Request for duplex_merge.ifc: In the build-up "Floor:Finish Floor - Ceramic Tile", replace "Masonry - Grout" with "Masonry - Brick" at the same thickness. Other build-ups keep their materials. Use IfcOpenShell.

First a look at what the model holds.

```python
import ifcopenshell
import ifcopenshell.util.element

model = ifcopenshell.open("duplex_merge.ifc")
print(model.schema)
for layer_set in model.by_type("IfcMaterialLayerSet"):
    if layer_set.LayerSetName == "Floor:Finish Floor - Ceramic Tile":
        for layer in layer_set.MaterialLayers:
            print(layer.id(), layer.Material and layer.Material.Name, layer.LayerThickness, sep=" | ")
        print(len(ifcopenshell.util.element.get_elements_by_material(model, layer_set)), "elements and types use it")
print(sorted(m.Name for m in model.by_type("IfcMaterial") if m.Name)[:60])
```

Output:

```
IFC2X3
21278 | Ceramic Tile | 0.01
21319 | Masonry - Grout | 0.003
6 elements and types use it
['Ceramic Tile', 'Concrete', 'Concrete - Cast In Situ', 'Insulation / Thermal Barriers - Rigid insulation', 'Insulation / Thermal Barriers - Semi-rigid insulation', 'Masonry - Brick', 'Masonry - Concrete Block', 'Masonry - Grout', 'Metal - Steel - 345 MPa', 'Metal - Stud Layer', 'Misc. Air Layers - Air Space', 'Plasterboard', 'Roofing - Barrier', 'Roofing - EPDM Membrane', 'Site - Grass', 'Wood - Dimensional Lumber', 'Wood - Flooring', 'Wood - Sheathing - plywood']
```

```python
import ifcopenshell
import ifcopenshell.api.material

model = ifcopenshell.open("duplex_merge.ifc")

layer_set = next(s for s in model.by_type("IfcMaterialLayerSet") if s.LayerSetName == "Floor:Finish Floor - Ceramic Tile")
layer = next(l for l in layer_set.MaterialLayers if l.Material and l.Material.Name == "Masonry - Grout")
material = next(m for m in model.by_type("IfcMaterial") if m.Name == "Masonry - Brick")

# Point this one layer at the other material; renaming the old one would change it everywhere.
ifcopenshell.api.material.edit_layer(model, layer=layer, attributes={}, material=material)

print([l.Material.Name if l.Material else None for l in layer_set.MaterialLayers])

model.write("duplex_merge-out.ifc")
```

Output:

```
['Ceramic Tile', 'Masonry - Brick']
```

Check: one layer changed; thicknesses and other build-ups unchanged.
